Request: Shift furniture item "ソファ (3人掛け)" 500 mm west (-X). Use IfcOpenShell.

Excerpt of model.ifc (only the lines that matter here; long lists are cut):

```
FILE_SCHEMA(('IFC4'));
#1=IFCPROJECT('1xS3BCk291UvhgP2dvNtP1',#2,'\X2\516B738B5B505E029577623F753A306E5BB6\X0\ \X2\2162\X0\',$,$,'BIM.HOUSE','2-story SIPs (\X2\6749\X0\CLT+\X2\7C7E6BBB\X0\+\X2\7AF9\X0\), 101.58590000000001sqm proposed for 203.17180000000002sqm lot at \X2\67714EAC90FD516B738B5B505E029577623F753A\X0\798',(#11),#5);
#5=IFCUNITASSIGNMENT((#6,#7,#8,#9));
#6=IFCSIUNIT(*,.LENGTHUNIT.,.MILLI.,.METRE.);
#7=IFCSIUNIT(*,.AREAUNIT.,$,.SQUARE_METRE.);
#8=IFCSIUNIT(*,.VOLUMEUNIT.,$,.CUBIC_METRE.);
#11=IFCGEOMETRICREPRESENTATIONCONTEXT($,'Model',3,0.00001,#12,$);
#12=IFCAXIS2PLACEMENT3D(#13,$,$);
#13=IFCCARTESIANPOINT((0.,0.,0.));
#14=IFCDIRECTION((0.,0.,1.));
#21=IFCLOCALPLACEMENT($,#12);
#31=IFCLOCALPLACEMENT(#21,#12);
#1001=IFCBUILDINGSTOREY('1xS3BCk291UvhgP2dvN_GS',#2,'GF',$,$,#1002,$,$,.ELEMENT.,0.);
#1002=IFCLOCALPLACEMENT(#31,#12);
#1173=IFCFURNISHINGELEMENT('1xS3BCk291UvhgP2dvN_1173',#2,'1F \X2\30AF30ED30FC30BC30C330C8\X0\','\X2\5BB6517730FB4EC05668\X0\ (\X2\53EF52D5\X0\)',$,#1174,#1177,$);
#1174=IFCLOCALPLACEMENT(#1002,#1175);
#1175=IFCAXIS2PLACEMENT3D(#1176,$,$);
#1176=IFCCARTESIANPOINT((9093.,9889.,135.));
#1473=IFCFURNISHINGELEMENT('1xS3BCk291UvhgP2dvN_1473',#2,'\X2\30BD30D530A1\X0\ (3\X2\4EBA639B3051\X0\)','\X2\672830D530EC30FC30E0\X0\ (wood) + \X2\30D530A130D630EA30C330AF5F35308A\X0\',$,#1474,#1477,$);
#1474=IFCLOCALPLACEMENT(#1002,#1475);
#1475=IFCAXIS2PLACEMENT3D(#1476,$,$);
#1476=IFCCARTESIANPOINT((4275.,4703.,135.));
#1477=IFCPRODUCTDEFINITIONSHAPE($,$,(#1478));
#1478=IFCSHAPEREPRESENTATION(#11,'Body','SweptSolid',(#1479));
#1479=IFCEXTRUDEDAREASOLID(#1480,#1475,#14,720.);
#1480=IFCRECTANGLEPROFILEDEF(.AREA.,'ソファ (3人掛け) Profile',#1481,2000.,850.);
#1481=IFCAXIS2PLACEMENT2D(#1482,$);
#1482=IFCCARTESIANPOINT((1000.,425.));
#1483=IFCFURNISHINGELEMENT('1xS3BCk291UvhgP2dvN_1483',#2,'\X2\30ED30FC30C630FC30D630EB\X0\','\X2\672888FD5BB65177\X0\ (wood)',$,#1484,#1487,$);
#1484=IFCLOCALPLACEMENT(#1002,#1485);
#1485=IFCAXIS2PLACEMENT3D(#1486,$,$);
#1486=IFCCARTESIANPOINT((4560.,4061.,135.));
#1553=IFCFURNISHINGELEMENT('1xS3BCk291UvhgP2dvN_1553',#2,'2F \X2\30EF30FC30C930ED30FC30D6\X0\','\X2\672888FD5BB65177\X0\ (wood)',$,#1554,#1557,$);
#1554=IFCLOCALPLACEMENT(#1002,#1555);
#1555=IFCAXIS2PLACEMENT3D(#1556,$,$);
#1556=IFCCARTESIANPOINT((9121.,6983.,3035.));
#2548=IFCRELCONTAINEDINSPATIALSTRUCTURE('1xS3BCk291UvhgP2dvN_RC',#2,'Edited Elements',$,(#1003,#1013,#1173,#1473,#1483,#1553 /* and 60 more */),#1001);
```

```python
import ifcopenshell
import ifcopenshell.api.geometry
import ifcopenshell.util.placement

model = ifcopenshell.open("model.ifc")

item = model.by_id(1473)
matrix = ifcopenshell.util.placement.get_local_placement(item.ObjectPlacement)
matrix[0, 3] -= 500.0
ifcopenshell.api.geometry.edit_object_placement(model, product=item, matrix=matrix, is_si=False)

print(ifcopenshell.util.placement.get_local_placement(item.ObjectPlacement).round(3) + 0.0)

model.write("model_edited.ifc")
```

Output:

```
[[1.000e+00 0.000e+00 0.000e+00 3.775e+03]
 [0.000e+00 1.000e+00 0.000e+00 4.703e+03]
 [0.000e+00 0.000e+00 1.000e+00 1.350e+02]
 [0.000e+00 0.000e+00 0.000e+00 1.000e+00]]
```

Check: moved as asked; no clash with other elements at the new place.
